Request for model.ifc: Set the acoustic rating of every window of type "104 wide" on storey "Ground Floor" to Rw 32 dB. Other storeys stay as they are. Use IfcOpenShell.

First a look at what the model holds.

```python
import ifcopenshell
import ifcopenshell.util.element

model = ifcopenshell.open("model.ifc")
print(model.schema)
storey = next(s for s in model.by_type("IfcBuildingStorey") if s.Name == "Ground Floor")
windows = [e for e in ifcopenshell.util.element.get_decomposition(storey) if e.is_a("IfcWindow")]
seen = {}
for e in windows:
    element_type = ifcopenshell.util.element.get_type(e)
    key = (element_type.Name if element_type != e and element_type else None, ifcopenshell.util.element.get_pset(e, "Pset_WindowCommon", "AcousticRating"))
    seen[key] = seen.get(key, 0) + 1
for (name, value), count in sorted(seen.items(), key=str):
    print(count, "x", name, "|", value)
```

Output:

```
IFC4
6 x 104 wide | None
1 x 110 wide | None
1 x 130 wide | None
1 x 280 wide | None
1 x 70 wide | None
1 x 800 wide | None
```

```python
import ifcopenshell
import ifcopenshell.api.pset
import ifcopenshell.util.element

model = ifcopenshell.open("model.ifc")

storey = next(s for s in model.by_type("IfcBuildingStorey") if s.Name == "Ground Floor")
windows = [e for e in ifcopenshell.util.element.get_decomposition(storey) if e.is_a("IfcWindow")]

count = 0
for e in windows:
    element_type = ifcopenshell.util.element.get_type(e)
    if element_type in (None, e) or element_type.Name != "104 wide":
        continue
    # add_pset returns the element's existing set when there is one.
    pset = ifcopenshell.api.pset.add_pset(model, product=e, name="Pset_WindowCommon")
    ifcopenshell.api.pset.edit_pset(model, pset=pset, properties={"AcousticRating": "Rw 32 dB"})
    count += 1

print(count, "windows updated")

model.write("model_rev.ifc")
```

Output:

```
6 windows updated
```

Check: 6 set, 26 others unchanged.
